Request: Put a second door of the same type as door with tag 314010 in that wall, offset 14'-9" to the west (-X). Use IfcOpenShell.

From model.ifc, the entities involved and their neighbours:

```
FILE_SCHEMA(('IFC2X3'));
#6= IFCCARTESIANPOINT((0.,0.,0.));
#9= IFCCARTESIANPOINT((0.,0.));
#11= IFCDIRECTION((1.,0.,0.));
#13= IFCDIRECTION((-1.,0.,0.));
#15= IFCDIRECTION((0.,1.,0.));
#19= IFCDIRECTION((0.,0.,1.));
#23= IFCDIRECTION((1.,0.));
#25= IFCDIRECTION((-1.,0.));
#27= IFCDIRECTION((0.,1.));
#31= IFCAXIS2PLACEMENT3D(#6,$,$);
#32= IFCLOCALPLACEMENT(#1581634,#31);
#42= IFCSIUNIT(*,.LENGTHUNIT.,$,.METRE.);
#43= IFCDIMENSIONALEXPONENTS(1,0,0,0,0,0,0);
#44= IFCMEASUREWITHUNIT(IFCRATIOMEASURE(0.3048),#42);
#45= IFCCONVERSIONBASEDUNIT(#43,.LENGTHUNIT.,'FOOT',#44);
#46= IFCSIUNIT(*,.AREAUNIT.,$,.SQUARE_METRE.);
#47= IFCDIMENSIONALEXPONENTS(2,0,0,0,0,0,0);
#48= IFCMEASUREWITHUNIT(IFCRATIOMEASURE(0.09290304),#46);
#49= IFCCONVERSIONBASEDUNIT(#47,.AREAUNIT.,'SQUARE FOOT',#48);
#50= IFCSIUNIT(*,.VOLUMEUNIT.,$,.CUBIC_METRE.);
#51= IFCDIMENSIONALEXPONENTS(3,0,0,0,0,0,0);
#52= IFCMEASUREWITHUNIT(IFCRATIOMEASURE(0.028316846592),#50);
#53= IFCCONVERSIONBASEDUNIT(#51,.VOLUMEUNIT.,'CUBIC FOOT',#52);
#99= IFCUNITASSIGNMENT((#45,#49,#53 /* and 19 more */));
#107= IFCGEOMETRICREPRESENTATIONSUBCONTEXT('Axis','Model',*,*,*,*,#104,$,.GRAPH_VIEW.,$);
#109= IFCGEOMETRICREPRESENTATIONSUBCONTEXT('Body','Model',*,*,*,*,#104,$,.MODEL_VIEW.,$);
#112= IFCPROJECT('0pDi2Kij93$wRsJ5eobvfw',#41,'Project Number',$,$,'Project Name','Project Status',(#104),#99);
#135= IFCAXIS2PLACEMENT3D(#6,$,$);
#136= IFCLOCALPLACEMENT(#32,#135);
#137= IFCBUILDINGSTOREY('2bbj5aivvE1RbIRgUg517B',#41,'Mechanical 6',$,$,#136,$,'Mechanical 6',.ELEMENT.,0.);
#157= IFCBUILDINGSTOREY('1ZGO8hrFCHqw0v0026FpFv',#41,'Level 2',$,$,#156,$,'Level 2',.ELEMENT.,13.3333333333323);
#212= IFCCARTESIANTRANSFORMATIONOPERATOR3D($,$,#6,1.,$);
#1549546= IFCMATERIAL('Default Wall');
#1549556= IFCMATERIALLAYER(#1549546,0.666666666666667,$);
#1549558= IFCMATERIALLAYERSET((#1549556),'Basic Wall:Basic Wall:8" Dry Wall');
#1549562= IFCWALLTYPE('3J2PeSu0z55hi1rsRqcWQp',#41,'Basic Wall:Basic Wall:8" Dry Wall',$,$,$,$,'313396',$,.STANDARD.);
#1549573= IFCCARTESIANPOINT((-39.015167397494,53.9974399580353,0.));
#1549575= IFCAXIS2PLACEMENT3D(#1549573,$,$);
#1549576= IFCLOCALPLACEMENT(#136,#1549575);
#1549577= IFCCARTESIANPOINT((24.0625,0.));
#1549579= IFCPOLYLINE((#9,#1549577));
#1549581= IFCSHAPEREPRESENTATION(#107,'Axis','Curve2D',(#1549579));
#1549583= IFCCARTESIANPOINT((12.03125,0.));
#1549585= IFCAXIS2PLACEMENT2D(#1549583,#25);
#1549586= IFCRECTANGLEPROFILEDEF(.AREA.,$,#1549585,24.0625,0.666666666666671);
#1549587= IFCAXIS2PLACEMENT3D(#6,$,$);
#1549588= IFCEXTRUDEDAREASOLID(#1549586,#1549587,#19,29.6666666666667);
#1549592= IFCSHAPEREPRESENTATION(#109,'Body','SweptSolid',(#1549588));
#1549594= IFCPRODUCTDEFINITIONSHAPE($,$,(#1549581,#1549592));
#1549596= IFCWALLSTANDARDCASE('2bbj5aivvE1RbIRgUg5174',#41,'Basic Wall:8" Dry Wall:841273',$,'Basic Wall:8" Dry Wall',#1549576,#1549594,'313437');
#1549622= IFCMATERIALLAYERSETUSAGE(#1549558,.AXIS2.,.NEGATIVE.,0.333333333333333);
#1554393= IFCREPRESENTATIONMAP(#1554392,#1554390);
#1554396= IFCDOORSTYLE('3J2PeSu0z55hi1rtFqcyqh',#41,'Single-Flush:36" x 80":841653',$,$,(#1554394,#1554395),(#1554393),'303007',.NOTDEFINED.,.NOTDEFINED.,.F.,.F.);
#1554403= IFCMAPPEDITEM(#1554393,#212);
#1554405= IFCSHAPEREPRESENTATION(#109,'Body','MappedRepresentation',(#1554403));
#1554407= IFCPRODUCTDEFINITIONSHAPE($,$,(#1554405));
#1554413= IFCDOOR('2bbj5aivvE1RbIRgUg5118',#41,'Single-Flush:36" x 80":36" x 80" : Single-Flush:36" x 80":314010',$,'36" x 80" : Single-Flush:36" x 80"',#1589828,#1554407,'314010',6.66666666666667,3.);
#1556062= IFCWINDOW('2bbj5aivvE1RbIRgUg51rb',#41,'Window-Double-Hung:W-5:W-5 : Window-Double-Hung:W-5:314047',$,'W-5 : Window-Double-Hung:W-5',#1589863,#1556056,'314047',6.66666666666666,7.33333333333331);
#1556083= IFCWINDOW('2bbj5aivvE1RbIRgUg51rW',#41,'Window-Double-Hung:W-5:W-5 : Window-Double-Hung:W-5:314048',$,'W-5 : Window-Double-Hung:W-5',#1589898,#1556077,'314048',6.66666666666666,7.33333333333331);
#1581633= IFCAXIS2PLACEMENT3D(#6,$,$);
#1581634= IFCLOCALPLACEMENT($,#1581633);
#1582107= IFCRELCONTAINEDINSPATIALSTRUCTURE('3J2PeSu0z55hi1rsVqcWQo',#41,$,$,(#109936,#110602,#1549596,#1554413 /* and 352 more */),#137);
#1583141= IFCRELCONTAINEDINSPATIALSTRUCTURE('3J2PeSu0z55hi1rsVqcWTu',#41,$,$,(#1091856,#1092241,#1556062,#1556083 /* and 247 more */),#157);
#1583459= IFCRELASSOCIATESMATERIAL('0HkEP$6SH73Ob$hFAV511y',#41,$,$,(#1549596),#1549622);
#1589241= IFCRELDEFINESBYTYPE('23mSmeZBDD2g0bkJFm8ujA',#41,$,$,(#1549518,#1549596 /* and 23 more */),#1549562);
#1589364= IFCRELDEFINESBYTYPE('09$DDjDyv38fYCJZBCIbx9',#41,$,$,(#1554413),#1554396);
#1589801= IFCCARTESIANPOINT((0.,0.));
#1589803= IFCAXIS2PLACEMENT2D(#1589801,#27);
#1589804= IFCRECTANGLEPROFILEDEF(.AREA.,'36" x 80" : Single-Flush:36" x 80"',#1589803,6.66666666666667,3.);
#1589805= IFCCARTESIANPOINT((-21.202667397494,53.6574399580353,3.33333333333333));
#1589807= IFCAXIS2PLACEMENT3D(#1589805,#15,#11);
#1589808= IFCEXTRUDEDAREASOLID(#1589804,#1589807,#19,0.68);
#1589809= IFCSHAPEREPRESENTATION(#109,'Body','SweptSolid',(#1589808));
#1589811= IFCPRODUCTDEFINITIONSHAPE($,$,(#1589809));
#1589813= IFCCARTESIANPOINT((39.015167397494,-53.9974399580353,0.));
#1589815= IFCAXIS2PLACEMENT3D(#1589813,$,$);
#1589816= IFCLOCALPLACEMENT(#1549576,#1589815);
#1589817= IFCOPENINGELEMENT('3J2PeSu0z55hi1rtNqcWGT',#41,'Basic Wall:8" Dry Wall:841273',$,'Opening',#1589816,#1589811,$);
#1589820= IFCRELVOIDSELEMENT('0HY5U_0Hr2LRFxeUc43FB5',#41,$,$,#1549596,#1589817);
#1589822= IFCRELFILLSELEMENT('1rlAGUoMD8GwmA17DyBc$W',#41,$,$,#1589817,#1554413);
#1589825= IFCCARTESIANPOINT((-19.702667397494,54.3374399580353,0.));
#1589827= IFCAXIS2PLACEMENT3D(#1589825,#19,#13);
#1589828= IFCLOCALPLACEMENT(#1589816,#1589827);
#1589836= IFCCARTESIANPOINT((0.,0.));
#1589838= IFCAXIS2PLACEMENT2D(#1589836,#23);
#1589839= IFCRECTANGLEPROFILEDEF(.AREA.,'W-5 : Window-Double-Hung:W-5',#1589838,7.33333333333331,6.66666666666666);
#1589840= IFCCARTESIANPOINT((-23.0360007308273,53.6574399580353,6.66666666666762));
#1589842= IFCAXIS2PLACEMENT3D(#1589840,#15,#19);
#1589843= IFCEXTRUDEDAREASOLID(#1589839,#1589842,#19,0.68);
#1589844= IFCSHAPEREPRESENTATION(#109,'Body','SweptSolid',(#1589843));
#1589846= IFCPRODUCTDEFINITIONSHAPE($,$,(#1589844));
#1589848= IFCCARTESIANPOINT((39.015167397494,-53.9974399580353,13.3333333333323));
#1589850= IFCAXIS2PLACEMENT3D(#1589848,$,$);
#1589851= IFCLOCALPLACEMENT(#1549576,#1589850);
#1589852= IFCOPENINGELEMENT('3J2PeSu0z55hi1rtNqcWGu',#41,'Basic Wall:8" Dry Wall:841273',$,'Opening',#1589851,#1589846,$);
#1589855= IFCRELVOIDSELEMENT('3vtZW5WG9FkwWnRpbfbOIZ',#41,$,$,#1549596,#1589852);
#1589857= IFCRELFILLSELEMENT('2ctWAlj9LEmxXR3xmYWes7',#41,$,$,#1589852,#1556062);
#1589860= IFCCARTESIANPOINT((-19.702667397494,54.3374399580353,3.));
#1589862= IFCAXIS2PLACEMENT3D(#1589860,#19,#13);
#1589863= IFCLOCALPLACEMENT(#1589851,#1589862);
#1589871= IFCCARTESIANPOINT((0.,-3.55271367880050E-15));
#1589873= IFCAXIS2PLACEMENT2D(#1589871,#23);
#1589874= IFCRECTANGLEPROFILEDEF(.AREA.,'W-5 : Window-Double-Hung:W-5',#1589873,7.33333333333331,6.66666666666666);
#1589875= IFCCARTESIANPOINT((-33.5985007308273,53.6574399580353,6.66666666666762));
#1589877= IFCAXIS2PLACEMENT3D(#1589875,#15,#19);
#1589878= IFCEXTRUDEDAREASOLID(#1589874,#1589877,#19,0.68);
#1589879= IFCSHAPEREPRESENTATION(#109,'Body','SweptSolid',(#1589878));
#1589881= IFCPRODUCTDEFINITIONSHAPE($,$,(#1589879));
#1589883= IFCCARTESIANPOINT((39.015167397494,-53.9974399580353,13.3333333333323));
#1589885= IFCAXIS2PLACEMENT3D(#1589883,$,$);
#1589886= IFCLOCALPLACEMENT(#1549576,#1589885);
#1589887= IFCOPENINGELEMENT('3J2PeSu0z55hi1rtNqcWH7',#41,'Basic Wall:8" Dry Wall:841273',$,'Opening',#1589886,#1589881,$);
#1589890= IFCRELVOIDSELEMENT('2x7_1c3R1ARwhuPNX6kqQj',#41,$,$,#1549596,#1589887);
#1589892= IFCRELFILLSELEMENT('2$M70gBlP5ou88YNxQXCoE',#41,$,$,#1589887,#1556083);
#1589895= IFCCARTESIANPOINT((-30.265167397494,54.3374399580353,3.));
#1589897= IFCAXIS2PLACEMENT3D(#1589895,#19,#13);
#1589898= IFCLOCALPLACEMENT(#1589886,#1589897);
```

```python
import ifcopenshell
import ifcopenshell.api.feature
import ifcopenshell.api.geometry
import ifcopenshell.api.root
import ifcopenshell.geom
import ifcopenshell.util.element
import ifcopenshell.util.placement
import ifcopenshell.util.shape
import ifcopenshell.util.unit

model = ifcopenshell.open("model.ifc")
unit_scale = ifcopenshell.util.unit.calculate_unit_scale(model)
settings = ifcopenshell.geom.settings()


def volume(element):
    """Net volume in cubic metres, openings subtracted."""
    shape = ifcopenshell.geom.create_shape(settings, element)
    return ifcopenshell.util.shape.get_volume(shape.geometry)


def reuse_history(source, copy):
    """copy_class also copies each property set's owner history, people and application; keep the originals."""
    for rel in copy.IsDefinedBy:
        if rel.is_a("IfcRelDefinesByProperties") and (history := rel.RelatingPropertyDefinition.OwnerHistory):
            rel.RelatingPropertyDefinition.OwnerHistory = source.OwnerHistory
            ifcopenshell.util.element.remove_deep2(model, history)


door = model.by_id(1554413)
opening = door.FillsVoids[0].RelatingOpeningElement
wall = opening.VoidsElements[0].RelatingBuildingElement
before = volume(wall)
shift = ifcopenshell.util.placement.get_local_placement(wall.ObjectPlacement)[:3, 0] * -177 * 0.0254 / unit_scale

# copy_class copies the void relationship, type, container and properties, but no geometry.
new_opening = ifcopenshell.api.root.copy_class(model, product=opening)
new_opening.Representation = ifcopenshell.util.element.copy_deep(
    model, opening.Representation, exclude=["IfcGeometricRepresentationContext", "IfcRepresentationMap"]
)
new_opening.Name = 'Basic Wall:8" Dry Wall'
new_door = ifcopenshell.api.root.copy_class(model, product=door)
new_door.Representation = ifcopenshell.util.element.copy_deep(
    model, door.Representation, exclude=["IfcGeometricRepresentationContext", "IfcRepresentationMap"]
)
new_door.Name = 'Single-Flush:36" x 80":36" x 80" : Single-Flush:36" x 80"'
new_door.Tag = None
reuse_history(door, new_door)
fills = ifcopenshell.api.feature.add_filling(model, opening=new_opening, element=new_door)
fills.OwnerHistory = new_door.OwnerHistory  # required in IFC2X3

for old, new in ((opening, new_opening), (door, new_door)):
    matrix = ifcopenshell.util.placement.get_local_placement(old.ObjectPlacement)
    matrix[:3, 3] += shift
    ifcopenshell.api.geometry.edit_object_placement(model, product=new, matrix=matrix, is_si=False)

after = volume(wall)

print(f"wall volume {before:.3f} -> {after:.3f} m3")

model.write("model_v2.ifc")
```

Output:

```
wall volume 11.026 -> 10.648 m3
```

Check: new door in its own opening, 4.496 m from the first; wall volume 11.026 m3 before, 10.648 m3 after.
